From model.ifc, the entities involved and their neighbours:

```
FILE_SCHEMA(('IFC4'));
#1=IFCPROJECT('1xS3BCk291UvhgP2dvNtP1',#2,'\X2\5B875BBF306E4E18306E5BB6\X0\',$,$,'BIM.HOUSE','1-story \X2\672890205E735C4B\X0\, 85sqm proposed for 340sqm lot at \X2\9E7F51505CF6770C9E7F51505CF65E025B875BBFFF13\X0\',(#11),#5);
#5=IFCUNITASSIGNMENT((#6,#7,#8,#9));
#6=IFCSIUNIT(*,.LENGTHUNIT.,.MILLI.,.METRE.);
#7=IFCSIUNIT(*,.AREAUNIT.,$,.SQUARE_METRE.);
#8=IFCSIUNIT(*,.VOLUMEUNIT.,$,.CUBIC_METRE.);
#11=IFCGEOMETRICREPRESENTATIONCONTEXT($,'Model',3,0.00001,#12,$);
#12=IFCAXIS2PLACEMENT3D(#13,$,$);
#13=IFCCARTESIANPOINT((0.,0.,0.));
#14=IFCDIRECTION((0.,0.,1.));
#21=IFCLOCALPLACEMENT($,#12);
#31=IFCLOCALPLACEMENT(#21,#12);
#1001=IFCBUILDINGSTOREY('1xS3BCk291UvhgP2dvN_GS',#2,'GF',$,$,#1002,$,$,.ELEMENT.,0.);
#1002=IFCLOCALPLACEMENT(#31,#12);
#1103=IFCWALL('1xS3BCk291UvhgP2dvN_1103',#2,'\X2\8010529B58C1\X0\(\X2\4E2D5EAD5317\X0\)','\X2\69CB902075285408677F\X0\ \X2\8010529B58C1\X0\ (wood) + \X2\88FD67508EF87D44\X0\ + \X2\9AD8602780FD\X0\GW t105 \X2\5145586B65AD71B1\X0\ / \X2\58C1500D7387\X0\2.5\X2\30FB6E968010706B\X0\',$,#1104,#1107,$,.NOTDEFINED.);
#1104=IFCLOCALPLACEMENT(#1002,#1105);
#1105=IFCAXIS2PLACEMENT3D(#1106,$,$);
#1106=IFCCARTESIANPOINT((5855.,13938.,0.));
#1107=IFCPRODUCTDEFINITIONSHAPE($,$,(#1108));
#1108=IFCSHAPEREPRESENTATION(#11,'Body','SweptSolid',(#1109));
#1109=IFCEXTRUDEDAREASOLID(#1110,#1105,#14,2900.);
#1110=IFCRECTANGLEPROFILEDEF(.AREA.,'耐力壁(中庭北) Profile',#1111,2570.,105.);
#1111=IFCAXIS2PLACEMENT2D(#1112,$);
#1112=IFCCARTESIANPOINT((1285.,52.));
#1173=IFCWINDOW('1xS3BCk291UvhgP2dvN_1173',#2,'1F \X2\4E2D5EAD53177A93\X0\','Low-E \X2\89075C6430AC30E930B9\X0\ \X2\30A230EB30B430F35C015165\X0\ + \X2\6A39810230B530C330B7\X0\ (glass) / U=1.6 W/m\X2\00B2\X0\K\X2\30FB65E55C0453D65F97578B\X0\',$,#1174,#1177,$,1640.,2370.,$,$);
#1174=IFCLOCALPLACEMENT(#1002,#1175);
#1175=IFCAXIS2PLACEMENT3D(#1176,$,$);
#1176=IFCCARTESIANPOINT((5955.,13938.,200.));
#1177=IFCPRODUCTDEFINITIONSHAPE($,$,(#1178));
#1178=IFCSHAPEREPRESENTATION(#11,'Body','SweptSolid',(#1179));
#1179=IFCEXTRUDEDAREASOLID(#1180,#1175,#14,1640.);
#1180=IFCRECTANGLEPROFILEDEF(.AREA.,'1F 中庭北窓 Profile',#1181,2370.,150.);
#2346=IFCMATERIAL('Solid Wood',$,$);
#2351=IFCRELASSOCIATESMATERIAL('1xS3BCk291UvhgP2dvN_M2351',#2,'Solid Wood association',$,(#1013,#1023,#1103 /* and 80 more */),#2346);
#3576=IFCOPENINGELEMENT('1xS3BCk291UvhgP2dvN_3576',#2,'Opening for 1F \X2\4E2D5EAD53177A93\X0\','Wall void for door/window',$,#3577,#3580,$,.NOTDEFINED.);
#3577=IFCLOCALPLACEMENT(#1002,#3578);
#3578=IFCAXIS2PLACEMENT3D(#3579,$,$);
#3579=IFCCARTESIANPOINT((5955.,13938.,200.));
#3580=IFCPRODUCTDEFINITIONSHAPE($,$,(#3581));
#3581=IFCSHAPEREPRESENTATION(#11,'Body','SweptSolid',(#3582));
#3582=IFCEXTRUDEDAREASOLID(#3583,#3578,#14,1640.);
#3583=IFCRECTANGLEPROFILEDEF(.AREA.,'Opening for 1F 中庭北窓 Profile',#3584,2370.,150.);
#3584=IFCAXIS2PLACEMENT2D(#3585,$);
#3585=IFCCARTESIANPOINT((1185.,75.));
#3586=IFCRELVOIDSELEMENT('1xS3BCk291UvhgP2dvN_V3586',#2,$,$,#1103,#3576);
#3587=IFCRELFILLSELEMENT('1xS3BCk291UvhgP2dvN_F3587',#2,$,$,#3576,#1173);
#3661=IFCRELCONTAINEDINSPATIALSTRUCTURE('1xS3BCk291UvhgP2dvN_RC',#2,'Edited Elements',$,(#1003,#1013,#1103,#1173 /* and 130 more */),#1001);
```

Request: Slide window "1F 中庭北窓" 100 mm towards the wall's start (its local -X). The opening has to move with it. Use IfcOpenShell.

```python
import ifcopenshell
import ifcopenshell.api.geometry
import ifcopenshell.util.placement
import ifcopenshell.util.unit

model = ifcopenshell.open("model.ifc")
unit_scale = ifcopenshell.util.unit.calculate_unit_scale(model)

window = model.by_guid("1xS3BCk291UvhgP2dvN_1173")
opening = window.FillsVoids[0].RelatingOpeningElement
wall = opening.VoidsElements[0].RelatingBuildingElement

wall_matrix = ifcopenshell.util.placement.get_local_placement(wall.ObjectPlacement)
shift = wall_matrix[:3, 0] * -0.1 / unit_scale
before = ifcopenshell.util.placement.get_local_placement(window.ObjectPlacement)[:3, 3].copy()

# The window is not placed relative to its opening, so move both.
for product in (opening, window):
    matrix = ifcopenshell.util.placement.get_local_placement(product.ObjectPlacement)
    matrix[:3, 3] += shift
    ifcopenshell.api.geometry.edit_object_placement(model, product=product, matrix=matrix, is_si=False)

after = ifcopenshell.util.placement.get_local_placement(window.ObjectPlacement)[:3, 3]
print("window moved by", (after - before).round(3) + 0.0)

model.write("model_v2.ifc")
```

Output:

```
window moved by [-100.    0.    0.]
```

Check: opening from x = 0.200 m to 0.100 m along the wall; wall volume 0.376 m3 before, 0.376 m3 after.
